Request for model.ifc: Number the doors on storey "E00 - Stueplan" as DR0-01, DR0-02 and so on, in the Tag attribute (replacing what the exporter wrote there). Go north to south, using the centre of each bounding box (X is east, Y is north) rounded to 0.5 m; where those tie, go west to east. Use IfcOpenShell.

First a look at what the model holds.

```python
import ifcopenshell
import ifcopenshell.util.element
import ifcopenshell.util.placement

model = ifcopenshell.open("model.ifc")
print(model.schema)
storey = next(s for s in model.by_type("IfcBuildingStorey") if s.Name == "E00 - Stueplan")
doors = [e for e in ifcopenshell.util.element.get_decomposition(storey) if e.is_a("IfcDoor")]
for e in sorted(doors, key=lambda e: e.id()):
    origin = ifcopenshell.util.placement.get_local_placement(e.ObjectPlacement)[:3, 3]
    print(e.id(), e.Tag, e.Name, origin.round(2) + 0.0, sep=" | ")
```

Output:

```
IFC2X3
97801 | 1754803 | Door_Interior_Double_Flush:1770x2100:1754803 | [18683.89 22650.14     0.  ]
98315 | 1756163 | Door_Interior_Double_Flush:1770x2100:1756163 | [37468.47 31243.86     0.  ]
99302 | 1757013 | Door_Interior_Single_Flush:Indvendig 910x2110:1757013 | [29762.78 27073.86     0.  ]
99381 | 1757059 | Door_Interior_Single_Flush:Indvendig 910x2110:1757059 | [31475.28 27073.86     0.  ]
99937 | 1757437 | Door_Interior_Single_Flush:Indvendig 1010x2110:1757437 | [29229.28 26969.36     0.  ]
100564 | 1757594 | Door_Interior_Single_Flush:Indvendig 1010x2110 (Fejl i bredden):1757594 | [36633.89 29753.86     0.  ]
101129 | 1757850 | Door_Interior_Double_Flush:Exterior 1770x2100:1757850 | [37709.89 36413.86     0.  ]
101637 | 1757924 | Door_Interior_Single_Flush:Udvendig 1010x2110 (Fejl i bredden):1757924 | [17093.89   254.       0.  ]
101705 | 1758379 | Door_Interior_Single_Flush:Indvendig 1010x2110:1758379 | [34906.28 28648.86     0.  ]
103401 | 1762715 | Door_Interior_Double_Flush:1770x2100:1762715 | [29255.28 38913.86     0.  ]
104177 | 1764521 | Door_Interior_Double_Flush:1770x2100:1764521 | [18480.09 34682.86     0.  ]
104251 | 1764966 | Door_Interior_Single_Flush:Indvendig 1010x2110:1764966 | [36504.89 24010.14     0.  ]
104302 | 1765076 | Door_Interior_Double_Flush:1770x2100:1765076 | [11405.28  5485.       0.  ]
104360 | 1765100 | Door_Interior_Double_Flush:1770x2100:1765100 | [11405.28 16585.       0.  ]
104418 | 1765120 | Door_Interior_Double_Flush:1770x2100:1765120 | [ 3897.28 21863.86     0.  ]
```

```python
import ifcopenshell
import ifcopenshell.geom
import ifcopenshell.util.element
import ifcopenshell.util.shape

model = ifcopenshell.open("model.ifc")
settings = ifcopenshell.geom.settings()
settings.set("use-world-coords", True)


def centre(element):
    shape = ifcopenshell.geom.create_shape(settings, element)
    return ifcopenshell.util.shape.get_bbox_centroid(shape.geometry)


storey = next(s for s in model.by_type("IfcBuildingStorey") if s.Name == "E00 - Stueplan")
doors = [e for e in ifcopenshell.util.element.get_decomposition(storey) if e.is_a("IfcDoor")]

# Insertion points can sit at a corner or the storey origin, so sort by the geometry (in metres).
centres = {e: centre(e) for e in doors}
doors.sort(key=lambda e: (-round(centres[e][1] / 0.5), centres[e][0]))

for i, e in enumerate(doors, start=1):
    number = f"DR0-{i:02d}"
    e.Tag = number
    print(e.id(), number)

model.write("model_rev.ifc")
```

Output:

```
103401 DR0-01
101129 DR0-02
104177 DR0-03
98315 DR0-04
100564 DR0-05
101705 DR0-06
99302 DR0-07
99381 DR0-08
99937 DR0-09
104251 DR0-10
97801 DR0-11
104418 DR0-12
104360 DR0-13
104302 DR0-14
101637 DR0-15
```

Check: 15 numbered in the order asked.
